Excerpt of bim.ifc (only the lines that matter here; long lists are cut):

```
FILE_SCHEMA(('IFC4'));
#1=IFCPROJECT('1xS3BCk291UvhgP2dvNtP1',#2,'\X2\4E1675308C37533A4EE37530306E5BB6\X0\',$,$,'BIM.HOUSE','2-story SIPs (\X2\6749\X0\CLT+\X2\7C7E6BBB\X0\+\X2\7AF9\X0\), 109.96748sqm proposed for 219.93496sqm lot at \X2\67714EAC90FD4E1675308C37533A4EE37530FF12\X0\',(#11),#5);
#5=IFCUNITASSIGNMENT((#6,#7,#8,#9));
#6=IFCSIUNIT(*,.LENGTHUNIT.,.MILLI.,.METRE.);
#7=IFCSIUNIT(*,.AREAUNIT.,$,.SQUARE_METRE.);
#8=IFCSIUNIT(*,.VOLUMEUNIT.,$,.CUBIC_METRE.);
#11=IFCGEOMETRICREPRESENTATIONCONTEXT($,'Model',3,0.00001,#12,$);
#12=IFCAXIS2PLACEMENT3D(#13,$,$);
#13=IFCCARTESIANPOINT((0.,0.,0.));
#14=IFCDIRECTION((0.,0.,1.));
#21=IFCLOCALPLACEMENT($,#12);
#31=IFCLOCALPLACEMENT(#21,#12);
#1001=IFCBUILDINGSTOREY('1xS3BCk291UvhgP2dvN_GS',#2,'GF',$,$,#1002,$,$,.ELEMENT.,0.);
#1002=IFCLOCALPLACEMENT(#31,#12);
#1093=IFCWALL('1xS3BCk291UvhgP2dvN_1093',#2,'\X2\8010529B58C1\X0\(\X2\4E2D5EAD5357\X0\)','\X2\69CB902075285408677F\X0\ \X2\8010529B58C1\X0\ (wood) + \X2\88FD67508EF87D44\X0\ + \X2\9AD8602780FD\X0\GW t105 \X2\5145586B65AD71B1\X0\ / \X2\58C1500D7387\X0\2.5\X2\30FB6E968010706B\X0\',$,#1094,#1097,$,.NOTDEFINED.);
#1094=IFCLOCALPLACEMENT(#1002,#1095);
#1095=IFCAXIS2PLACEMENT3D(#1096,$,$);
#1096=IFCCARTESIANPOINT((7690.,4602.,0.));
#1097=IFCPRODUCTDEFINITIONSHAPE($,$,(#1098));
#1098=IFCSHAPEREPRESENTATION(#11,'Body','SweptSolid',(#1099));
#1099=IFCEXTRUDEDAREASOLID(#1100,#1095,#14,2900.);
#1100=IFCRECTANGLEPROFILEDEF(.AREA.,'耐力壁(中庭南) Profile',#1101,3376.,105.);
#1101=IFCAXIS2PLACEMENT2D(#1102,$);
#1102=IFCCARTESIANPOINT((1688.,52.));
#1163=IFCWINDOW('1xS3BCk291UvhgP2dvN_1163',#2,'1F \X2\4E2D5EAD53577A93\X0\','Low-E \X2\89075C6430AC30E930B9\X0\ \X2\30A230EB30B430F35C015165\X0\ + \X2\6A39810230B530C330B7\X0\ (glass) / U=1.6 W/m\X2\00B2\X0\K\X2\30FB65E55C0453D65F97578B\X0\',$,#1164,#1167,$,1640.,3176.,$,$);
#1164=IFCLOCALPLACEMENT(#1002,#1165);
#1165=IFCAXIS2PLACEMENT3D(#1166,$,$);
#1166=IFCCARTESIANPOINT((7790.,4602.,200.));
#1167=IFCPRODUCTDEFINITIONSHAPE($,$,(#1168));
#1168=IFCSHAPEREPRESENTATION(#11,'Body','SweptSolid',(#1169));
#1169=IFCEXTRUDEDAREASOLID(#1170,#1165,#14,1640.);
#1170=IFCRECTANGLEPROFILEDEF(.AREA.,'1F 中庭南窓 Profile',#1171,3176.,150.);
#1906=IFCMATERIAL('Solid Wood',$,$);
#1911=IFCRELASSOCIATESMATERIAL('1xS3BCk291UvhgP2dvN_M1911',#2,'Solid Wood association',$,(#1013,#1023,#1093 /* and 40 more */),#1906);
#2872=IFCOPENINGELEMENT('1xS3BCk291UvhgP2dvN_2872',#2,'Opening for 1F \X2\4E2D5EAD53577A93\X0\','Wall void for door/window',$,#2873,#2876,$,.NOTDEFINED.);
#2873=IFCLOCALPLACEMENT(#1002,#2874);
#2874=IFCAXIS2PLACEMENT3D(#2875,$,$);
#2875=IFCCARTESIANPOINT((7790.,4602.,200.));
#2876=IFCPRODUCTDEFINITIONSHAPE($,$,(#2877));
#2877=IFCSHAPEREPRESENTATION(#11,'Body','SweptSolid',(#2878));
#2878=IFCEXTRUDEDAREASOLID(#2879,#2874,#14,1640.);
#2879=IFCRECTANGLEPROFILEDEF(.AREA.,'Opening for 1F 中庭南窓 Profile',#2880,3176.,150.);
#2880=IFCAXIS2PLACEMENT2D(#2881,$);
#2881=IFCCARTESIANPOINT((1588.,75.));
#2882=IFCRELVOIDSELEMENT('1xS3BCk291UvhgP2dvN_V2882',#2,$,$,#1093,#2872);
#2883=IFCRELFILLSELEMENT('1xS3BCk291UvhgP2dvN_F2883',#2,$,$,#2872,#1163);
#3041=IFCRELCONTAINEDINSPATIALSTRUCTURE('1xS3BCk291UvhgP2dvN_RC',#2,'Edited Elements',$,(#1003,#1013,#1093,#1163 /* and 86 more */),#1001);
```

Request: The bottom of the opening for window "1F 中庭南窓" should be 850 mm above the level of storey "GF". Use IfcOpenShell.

```python
import numpy as np
import ifcopenshell
import ifcopenshell.api.geometry
import ifcopenshell.geom
import ifcopenshell.util.element
import ifcopenshell.util.placement
import ifcopenshell.util.shape
import ifcopenshell.util.unit

model = ifcopenshell.open("bim.ifc")
unit_scale = ifcopenshell.util.unit.calculate_unit_scale(model)

window = model.by_guid("1xS3BCk291UvhgP2dvN_1163")
opening = window.FillsVoids[0].RelatingOpeningElement
storey = ifcopenshell.util.element.get_container(window, ifc_class="IfcBuildingStorey")
level = ifcopenshell.util.placement.get_local_placement(storey.ObjectPlacement)[2, 3]

# The opening's origin need not be at the sill, so measure its lowest point.
shape = ifcopenshell.geom.create_shape(ifcopenshell.geom.settings(), opening)
bottom = ifcopenshell.util.shape.get_shape_bottom_elevation(shape, shape.geometry) / unit_scale
dz = level + 850.0 - bottom

shift = np.array([0.0, 0.0, dz])
# The window is not placed relative to its opening, so move both.
for product in (opening, window):
    matrix = ifcopenshell.util.placement.get_local_placement(product.ObjectPlacement)
    matrix[:3, 3] += shift
    ifcopenshell.api.geometry.edit_object_placement(model, product=product, matrix=matrix, is_si=False)

print(f"moved by {dz * unit_scale:+.3f} m")

model.write("bim_updated.ifc")
```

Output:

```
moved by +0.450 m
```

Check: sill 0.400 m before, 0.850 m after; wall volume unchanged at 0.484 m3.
